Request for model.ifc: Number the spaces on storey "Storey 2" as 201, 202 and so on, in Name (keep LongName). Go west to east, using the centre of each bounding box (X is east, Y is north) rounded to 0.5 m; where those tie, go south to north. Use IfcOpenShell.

First a look at what the model holds.

```python
import ifcopenshell
import ifcopenshell.util.element
import ifcopenshell.util.placement

model = ifcopenshell.open("model.ifc")
print(model.schema)
storey = next(s for s in model.by_type("IfcBuildingStorey") if s.Name == "Storey 2")
spaces = [e for e in ifcopenshell.util.element.get_decomposition(storey) if e.is_a("IfcSpace")]
for e in sorted(spaces, key=lambda e: e.id()):
    origin = ifcopenshell.util.placement.get_local_placement(e.ObjectPlacement)[:3, 3]
    print(e.id(), e.Name, e.LongName, origin.round(2) + 0.0, sep=" | ")
```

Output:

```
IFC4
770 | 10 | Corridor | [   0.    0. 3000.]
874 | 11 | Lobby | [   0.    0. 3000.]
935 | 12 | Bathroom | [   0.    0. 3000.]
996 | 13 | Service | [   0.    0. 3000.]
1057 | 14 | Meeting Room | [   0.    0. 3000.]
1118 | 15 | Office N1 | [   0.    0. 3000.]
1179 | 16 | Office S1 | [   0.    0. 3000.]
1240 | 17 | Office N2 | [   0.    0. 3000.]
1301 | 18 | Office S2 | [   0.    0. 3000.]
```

```python
import ifcopenshell
import ifcopenshell.geom
import ifcopenshell.util.element
import ifcopenshell.util.shape

model = ifcopenshell.open("model.ifc")
settings = ifcopenshell.geom.settings()
settings.set("use-world-coords", True)


def centre(element):
    shape = ifcopenshell.geom.create_shape(settings, element)
    return ifcopenshell.util.shape.get_bbox_centroid(shape.geometry)


storey = next(s for s in model.by_type("IfcBuildingStorey") if s.Name == "Storey 2")
spaces = [e for e in ifcopenshell.util.element.get_decomposition(storey) if e.is_a("IfcSpace")]

# Insertion points can sit at a corner or the storey origin, so sort by the geometry (in metres).
centres = {e: centre(e) for e in spaces}
spaces.sort(key=lambda e: (round(centres[e][0] / 0.5), centres[e][1]))

for i, e in enumerate(spaces, start=1):
    number = f"2{i:02d}"
    e.Name = number
    print(e.id(), number)

model.write("model_rev.ifc")
```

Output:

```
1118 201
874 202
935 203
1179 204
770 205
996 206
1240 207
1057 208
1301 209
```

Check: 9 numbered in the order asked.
